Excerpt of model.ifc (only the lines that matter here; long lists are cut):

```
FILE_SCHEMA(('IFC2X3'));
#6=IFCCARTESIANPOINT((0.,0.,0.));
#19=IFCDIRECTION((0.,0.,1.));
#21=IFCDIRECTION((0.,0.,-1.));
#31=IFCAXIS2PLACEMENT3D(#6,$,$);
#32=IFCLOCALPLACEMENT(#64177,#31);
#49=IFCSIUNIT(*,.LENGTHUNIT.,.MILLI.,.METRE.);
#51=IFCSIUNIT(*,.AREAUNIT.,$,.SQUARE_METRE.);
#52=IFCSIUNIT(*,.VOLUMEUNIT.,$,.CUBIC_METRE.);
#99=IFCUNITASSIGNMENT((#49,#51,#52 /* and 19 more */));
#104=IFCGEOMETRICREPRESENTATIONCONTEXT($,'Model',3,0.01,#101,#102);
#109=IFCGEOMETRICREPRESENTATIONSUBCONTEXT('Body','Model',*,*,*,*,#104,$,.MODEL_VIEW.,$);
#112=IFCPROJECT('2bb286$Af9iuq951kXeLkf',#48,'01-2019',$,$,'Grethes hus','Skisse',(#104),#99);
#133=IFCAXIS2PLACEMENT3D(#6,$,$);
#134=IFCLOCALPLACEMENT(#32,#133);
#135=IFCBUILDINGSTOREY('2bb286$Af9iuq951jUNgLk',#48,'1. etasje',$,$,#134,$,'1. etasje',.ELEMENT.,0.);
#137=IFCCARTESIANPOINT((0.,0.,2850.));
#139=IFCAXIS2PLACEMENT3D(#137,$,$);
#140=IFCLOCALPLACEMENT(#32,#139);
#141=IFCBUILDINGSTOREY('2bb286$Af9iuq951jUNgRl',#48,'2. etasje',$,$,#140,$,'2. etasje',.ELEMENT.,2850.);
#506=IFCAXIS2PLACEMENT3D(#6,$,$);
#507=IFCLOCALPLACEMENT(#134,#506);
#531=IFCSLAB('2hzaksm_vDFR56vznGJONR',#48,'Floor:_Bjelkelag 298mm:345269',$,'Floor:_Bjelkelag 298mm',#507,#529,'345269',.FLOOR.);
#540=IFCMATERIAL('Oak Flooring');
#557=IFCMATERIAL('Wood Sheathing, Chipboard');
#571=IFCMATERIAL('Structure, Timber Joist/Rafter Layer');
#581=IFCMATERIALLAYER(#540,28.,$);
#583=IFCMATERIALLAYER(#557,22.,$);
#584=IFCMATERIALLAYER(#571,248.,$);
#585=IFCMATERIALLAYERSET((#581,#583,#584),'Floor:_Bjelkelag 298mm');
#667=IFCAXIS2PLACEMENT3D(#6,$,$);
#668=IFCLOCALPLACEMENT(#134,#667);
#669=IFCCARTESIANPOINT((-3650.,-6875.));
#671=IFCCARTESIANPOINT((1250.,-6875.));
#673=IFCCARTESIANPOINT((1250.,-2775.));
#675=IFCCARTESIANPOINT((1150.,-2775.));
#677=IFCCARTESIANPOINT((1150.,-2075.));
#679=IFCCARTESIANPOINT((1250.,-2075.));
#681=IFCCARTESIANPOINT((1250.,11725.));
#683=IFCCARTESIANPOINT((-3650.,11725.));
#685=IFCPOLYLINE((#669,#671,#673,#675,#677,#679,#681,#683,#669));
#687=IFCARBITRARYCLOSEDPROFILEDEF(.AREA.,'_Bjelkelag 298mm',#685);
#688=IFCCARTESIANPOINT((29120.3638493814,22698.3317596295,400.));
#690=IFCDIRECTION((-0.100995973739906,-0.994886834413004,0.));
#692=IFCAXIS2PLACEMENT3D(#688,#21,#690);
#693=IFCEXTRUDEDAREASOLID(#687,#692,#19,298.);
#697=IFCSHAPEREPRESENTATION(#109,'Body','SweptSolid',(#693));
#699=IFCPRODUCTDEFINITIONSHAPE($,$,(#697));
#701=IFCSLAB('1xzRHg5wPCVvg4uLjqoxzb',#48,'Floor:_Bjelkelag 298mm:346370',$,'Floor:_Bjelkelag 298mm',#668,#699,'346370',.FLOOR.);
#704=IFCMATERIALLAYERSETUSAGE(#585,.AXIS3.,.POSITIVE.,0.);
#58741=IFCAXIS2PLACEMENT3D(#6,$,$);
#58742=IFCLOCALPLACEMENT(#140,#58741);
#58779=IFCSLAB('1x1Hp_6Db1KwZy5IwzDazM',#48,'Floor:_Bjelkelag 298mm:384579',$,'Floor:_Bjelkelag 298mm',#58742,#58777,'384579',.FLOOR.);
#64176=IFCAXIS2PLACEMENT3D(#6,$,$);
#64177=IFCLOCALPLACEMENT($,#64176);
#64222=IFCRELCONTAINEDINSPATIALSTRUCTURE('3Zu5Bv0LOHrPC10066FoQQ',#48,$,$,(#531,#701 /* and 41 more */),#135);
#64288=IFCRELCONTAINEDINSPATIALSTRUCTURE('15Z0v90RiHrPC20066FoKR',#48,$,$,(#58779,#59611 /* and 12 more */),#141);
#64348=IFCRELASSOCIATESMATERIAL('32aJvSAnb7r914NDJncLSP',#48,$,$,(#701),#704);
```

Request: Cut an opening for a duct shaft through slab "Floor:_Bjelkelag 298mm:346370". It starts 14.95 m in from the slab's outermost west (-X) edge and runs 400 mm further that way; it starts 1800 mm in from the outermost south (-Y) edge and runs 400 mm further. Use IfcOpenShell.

```python
import numpy as np
import ifcopenshell
import ifcopenshell.api.feature
import ifcopenshell.api.geometry
import ifcopenshell.api.root
import ifcopenshell.geom
import ifcopenshell.util.placement
import ifcopenshell.util.representation
import ifcopenshell.util.shape
import ifcopenshell.util.unit

model = ifcopenshell.open("model.ifc")
unit_scale = ifcopenshell.util.unit.calculate_unit_scale(model)
settings = ifcopenshell.geom.settings()


def volume(element):
    """Net volume in cubic metres, openings subtracted."""
    shape = ifcopenshell.geom.create_shape(settings, element)
    return ifcopenshell.util.shape.get_volume(shape.geometry)


slab = model.by_guid("1xzRHg5wPCVvg4uLjqoxzb")
before = volume(slab)

# Extent in the slab's own axes, in metres. The edges named are its -X and -Y sides.
slab_shape = ifcopenshell.geom.create_shape(settings, slab)
vertices = ifcopenshell.util.shape.get_vertices(slab_shape.geometry)
x_min, y_min, bottom = vertices.min(axis=0)
top = vertices[:, 2].max()

opening = ifcopenshell.api.root.create_entity(model, ifc_class="IfcOpeningElement", name="Duct shaft opening")
context = ifcopenshell.util.representation.get_context(model, "Model", "Body", "MODEL_VIEW")
width, depth = 0.4, 0.4
outline = [(0.0, 0.0), (width, 0.0), (width, depth), (0.0, depth), (0.0, 0.0)]
# Overshoot both faces by 50 mm so the cut is clean.
shape = ifcopenshell.api.geometry.add_slab_representation(
    model, context=context, depth=top - bottom + 0.1, polyline=outline
)
ifcopenshell.api.geometry.assign_representation(model, product=opening, representation=shape)

matrix = ifcopenshell.util.placement.get_local_placement(slab.ObjectPlacement)
matrix[:, 3] = matrix @ np.append(np.array([x_min + 14.95, y_min + 1.8, bottom - 0.05]) / unit_scale, 1.0)
ifcopenshell.api.geometry.edit_object_placement(model, product=opening, matrix=matrix, is_si=False)
ifcopenshell.api.feature.add_feature(model, feature=opening, element=slab)

after = volume(slab)

print(f"slab volume {before:.3f} -> {after:.3f} m3")

model.write("model-out.ifc")
```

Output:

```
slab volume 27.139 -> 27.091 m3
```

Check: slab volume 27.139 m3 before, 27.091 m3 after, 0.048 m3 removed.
